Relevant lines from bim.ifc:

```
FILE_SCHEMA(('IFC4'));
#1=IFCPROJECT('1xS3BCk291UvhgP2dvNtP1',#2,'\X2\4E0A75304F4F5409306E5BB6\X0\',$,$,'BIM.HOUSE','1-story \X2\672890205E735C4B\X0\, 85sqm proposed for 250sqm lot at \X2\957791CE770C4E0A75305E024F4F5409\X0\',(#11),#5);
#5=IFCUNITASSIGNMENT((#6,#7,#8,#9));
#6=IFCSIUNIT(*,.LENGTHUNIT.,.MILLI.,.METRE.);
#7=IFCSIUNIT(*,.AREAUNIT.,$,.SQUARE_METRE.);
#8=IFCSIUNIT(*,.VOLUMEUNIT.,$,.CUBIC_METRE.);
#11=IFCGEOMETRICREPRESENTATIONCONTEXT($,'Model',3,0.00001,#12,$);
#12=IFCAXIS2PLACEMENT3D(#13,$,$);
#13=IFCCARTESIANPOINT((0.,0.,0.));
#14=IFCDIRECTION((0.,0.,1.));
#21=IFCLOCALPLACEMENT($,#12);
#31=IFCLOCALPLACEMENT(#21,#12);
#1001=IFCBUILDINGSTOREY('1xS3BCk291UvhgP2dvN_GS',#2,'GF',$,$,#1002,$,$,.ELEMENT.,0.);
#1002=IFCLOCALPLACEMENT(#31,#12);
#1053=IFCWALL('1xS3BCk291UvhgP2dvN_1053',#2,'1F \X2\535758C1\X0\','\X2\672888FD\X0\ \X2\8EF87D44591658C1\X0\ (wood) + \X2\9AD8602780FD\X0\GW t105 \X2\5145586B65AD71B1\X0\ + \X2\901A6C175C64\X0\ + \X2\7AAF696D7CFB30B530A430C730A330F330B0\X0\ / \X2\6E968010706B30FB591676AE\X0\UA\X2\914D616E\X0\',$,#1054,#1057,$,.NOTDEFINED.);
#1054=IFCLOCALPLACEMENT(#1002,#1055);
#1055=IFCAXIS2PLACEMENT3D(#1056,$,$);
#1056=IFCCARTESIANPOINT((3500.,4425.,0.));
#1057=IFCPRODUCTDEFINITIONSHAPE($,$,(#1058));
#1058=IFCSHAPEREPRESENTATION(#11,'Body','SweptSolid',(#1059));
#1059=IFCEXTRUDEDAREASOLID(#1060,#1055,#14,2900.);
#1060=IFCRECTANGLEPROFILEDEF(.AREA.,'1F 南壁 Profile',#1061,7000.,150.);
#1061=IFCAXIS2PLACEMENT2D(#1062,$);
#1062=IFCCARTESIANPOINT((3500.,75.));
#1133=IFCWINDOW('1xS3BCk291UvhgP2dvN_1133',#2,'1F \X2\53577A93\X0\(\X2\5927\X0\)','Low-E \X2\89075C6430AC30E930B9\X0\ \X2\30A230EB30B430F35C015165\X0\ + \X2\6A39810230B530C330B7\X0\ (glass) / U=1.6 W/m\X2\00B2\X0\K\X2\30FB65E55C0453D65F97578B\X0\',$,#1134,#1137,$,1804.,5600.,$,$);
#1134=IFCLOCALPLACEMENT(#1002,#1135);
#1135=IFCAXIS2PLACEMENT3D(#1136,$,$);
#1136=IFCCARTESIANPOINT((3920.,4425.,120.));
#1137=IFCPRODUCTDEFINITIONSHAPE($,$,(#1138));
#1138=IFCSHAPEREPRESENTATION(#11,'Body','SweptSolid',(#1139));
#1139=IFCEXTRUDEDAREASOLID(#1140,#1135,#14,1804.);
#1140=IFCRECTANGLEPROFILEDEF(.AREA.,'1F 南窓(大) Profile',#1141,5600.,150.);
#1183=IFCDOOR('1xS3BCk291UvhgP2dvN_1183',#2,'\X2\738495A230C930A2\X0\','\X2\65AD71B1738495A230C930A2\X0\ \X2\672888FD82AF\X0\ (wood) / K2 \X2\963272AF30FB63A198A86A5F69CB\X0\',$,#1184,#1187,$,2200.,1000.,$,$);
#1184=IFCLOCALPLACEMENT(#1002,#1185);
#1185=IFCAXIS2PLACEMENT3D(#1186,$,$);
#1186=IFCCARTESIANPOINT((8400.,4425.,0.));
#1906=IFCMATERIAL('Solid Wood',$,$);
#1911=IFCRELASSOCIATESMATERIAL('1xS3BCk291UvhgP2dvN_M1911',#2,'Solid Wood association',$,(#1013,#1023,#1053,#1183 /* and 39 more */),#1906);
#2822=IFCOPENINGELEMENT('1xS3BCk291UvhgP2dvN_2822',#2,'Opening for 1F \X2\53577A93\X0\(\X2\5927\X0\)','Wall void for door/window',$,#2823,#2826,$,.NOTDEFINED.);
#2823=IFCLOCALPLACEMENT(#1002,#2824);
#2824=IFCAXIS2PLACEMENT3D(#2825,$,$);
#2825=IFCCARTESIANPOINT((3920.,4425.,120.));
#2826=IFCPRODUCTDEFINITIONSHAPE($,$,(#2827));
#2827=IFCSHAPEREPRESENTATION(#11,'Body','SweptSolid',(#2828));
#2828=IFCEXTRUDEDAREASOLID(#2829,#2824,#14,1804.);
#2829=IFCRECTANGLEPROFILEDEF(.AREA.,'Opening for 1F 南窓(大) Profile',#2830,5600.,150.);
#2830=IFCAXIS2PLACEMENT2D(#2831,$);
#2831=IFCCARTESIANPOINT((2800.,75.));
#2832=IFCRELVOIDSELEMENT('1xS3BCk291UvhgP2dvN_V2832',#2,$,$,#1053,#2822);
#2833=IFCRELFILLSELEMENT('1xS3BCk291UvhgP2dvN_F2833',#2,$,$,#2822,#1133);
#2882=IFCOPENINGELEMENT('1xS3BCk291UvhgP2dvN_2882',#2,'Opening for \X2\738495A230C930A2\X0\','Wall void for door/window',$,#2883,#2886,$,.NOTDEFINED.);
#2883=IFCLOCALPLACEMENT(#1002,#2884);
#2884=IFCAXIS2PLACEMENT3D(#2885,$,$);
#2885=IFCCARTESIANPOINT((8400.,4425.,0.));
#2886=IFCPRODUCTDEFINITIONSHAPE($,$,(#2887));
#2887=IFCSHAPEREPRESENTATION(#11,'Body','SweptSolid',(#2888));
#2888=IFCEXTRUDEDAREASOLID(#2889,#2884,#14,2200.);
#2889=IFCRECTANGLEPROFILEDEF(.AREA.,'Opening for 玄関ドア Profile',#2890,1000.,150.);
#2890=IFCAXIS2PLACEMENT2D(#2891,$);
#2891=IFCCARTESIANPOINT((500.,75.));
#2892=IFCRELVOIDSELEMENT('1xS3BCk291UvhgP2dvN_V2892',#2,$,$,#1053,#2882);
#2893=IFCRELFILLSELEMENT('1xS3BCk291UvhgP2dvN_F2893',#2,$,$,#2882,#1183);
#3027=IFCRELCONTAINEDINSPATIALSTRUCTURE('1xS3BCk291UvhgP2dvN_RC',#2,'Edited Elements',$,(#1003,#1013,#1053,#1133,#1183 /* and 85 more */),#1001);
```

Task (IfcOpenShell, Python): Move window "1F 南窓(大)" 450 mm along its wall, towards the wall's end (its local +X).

```python
import ifcopenshell
import ifcopenshell.api.geometry
import ifcopenshell.util.placement
import ifcopenshell.util.unit

model = ifcopenshell.open("bim.ifc")
unit_scale = ifcopenshell.util.unit.calculate_unit_scale(model)

window = model.by_guid("1xS3BCk291UvhgP2dvN_1133")
opening = window.FillsVoids[0].RelatingOpeningElement
wall = opening.VoidsElements[0].RelatingBuildingElement

wall_matrix = ifcopenshell.util.placement.get_local_placement(wall.ObjectPlacement)
shift = wall_matrix[:3, 0] * 0.45 / unit_scale
before = ifcopenshell.util.placement.get_local_placement(window.ObjectPlacement)[:3, 3].copy()

# The window is not placed relative to its opening, so move both.
for product in (opening, window):
    matrix = ifcopenshell.util.placement.get_local_placement(product.ObjectPlacement)
    matrix[:3, 3] += shift
    ifcopenshell.api.geometry.edit_object_placement(model, product=product, matrix=matrix, is_si=False)

after = ifcopenshell.util.placement.get_local_placement(window.ObjectPlacement)[:3, 3]
print("window moved by", (after - before).round(3) + 0.0)

model.write("bim-out.ifc")
```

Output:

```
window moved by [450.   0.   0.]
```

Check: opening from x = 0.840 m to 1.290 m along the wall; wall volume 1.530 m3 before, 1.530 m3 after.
